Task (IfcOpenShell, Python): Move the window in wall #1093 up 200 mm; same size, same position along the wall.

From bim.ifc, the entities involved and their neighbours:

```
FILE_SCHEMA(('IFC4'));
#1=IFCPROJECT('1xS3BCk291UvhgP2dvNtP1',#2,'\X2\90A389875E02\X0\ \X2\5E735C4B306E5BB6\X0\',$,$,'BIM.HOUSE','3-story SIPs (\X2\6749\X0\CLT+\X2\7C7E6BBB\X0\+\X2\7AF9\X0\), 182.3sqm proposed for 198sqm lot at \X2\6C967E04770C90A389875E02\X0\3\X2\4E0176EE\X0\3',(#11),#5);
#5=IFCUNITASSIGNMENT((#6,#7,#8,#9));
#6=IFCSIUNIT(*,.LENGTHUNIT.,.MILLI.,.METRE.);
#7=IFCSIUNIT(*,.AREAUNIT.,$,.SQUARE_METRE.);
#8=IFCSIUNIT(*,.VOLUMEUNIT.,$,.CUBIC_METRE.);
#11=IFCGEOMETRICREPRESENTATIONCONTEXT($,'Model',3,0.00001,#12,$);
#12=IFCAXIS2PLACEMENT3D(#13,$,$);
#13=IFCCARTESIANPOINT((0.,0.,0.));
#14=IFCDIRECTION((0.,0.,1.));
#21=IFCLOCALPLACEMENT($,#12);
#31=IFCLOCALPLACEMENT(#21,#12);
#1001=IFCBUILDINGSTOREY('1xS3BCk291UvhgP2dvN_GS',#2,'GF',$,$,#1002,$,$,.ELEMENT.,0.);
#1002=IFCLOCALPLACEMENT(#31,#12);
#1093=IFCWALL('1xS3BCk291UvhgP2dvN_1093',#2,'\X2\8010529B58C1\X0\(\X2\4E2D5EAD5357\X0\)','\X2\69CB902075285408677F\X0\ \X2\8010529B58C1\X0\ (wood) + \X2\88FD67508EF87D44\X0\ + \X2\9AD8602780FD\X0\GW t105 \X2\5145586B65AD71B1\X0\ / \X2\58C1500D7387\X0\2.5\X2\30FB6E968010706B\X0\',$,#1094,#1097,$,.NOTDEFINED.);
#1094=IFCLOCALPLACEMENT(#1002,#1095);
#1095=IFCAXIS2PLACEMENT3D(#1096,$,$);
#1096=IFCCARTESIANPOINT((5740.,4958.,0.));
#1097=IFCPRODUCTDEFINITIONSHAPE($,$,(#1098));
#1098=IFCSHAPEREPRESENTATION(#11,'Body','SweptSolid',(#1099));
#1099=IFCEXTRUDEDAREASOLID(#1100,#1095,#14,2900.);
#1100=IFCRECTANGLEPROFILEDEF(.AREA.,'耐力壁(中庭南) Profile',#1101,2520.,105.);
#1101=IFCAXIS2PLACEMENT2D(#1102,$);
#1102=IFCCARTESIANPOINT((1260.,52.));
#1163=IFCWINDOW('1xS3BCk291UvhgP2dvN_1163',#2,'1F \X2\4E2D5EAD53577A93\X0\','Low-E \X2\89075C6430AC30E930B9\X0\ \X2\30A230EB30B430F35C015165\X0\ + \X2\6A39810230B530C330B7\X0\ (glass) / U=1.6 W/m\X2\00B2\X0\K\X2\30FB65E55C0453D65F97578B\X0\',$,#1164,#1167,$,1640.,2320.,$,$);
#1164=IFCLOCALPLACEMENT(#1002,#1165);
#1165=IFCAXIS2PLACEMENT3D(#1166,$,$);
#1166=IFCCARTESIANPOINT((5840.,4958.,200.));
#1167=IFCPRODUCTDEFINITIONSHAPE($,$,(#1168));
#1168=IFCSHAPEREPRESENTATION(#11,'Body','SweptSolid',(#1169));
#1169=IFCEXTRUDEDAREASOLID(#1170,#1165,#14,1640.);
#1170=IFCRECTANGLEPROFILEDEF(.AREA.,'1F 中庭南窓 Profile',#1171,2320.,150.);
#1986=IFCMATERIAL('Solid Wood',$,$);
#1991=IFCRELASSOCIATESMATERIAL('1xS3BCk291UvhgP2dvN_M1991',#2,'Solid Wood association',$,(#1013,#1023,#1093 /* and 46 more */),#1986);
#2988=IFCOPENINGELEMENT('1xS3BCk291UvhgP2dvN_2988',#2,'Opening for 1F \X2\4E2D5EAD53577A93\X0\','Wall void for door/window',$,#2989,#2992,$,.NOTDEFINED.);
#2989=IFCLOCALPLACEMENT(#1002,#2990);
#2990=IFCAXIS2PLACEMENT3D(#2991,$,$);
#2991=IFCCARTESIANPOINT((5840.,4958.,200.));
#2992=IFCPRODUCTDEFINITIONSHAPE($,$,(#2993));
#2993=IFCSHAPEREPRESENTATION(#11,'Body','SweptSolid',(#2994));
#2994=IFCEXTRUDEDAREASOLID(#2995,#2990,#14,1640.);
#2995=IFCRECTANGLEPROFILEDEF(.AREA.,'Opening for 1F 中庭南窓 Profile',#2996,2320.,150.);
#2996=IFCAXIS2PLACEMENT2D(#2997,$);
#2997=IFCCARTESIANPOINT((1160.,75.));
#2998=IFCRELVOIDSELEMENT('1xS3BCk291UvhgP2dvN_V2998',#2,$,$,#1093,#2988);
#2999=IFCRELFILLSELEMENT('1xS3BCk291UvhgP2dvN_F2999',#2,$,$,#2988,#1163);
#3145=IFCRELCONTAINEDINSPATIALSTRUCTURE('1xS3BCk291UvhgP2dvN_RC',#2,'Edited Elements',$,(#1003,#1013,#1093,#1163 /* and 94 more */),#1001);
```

```python
import numpy as np
import ifcopenshell
import ifcopenshell.api.geometry
import ifcopenshell.util.placement
import ifcopenshell.util.unit

model = ifcopenshell.open("bim.ifc")
unit_scale = ifcopenshell.util.unit.calculate_unit_scale(model)

window = model.by_guid("1xS3BCk291UvhgP2dvN_1163")
opening = window.FillsVoids[0].RelatingOpeningElement
dz = 0.2 / unit_scale

shift = np.array([0.0, 0.0, dz])
# The window is not placed relative to its opening, so move both.
for product in (opening, window):
    matrix = ifcopenshell.util.placement.get_local_placement(product.ObjectPlacement)
    matrix[:3, 3] += shift
    ifcopenshell.api.geometry.edit_object_placement(model, product=product, matrix=matrix, is_si=False)

print(f"moved by {dz * unit_scale:+.3f} m")

model.write("bim_updated.ifc")
```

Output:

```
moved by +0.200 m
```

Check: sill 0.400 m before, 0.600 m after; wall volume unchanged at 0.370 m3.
